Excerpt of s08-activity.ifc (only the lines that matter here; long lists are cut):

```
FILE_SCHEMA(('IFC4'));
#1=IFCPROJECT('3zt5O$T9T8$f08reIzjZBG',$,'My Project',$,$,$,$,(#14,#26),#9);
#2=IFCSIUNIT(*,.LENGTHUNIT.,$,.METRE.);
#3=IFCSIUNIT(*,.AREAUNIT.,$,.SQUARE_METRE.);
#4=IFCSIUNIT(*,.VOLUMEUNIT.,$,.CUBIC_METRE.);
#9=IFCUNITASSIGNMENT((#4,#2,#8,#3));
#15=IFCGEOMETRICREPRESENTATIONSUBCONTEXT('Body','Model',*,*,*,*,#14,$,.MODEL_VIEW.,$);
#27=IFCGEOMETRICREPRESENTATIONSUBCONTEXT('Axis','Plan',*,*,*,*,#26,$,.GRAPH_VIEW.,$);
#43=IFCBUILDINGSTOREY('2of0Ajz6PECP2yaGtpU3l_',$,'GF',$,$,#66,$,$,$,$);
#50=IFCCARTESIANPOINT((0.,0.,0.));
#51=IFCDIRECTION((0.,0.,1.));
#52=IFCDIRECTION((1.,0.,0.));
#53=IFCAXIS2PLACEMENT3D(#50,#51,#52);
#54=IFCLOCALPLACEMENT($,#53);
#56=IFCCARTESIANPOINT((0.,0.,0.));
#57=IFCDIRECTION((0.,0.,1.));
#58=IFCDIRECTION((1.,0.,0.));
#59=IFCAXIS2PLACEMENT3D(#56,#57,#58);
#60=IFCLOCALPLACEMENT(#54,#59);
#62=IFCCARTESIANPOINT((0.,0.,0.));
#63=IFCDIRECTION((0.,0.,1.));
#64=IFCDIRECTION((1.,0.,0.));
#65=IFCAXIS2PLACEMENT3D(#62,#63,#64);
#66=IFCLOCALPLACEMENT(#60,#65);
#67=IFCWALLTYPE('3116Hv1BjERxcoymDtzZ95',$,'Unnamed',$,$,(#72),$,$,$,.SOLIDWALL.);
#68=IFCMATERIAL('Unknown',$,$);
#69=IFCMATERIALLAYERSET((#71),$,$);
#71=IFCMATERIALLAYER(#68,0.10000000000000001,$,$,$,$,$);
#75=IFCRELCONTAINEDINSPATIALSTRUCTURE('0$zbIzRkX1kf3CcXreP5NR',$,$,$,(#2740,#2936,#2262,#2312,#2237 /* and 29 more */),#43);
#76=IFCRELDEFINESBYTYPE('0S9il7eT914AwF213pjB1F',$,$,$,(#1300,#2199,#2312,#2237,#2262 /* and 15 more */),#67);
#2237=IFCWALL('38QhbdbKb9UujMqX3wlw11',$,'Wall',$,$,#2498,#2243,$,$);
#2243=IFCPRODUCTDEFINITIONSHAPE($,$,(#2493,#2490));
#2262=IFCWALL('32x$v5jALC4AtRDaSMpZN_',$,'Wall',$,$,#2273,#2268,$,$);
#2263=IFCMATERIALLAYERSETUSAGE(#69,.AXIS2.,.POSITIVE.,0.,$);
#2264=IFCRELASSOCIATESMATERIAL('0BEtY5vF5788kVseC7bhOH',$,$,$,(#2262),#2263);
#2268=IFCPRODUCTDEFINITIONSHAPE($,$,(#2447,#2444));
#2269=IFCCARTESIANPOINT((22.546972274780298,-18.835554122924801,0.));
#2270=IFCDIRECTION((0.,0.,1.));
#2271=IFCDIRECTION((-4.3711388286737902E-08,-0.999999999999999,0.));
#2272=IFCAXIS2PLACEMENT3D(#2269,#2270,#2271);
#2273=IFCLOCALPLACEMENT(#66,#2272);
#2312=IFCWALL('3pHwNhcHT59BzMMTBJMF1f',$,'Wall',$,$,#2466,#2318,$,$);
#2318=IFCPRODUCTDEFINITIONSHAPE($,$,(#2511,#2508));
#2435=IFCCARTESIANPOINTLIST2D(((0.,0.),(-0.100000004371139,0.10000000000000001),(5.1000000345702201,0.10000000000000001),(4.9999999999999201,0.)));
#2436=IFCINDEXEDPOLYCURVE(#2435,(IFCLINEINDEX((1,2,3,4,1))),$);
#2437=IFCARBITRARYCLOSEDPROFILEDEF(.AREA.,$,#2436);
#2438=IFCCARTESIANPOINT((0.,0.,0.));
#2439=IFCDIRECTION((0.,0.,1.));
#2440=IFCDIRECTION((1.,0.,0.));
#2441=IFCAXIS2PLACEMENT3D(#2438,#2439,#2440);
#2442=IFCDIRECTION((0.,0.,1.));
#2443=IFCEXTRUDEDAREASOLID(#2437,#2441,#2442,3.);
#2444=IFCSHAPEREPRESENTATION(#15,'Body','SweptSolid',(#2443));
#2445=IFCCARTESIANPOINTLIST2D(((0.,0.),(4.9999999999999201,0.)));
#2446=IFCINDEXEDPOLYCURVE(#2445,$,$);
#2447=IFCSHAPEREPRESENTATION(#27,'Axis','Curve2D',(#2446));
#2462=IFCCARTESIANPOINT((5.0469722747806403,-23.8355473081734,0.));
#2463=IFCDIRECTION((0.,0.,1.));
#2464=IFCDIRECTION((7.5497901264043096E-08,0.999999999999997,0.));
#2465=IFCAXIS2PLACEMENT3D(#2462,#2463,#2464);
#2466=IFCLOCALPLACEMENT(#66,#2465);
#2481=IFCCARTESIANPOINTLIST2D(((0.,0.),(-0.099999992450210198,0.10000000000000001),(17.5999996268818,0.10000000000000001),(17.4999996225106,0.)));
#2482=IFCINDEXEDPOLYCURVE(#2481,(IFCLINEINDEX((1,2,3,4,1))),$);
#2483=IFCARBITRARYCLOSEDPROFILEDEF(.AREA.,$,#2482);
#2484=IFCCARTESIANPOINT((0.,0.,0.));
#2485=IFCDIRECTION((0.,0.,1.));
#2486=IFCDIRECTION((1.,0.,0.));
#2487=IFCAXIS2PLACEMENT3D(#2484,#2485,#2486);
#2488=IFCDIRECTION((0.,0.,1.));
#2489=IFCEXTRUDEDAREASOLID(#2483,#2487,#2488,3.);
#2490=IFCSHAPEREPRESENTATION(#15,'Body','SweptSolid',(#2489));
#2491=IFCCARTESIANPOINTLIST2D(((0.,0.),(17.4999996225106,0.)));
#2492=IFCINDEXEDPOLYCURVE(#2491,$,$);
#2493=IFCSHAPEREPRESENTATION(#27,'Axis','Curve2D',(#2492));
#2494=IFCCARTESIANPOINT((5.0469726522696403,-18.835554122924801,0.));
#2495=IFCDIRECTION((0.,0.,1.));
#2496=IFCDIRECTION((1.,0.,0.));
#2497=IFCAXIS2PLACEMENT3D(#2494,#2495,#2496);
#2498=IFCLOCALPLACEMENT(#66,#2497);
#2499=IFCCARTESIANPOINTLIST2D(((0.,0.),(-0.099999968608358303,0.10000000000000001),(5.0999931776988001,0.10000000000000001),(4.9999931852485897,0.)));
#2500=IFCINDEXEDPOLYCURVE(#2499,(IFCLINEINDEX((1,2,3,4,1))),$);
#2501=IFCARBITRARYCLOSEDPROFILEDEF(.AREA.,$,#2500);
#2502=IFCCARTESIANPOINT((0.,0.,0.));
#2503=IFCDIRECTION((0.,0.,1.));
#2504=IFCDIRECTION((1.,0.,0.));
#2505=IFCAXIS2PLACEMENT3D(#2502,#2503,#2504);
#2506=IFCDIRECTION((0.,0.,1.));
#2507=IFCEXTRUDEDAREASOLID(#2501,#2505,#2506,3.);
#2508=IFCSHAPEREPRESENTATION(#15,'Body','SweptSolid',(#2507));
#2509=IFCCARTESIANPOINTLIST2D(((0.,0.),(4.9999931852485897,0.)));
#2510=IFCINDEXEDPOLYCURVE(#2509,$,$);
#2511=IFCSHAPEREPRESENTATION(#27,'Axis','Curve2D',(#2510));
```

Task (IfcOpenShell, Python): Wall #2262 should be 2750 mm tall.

```python
import ifcopenshell
import ifcopenshell.geom
import ifcopenshell.util.representation
import ifcopenshell.util.shape
import ifcopenshell.util.unit

model = ifcopenshell.open("s08-activity.ifc")
unit_scale = ifcopenshell.util.unit.calculate_unit_scale(model)
settings = ifcopenshell.geom.settings()


def volume(element):
    """Net volume in cubic metres, openings subtracted."""
    shape = ifcopenshell.geom.create_shape(settings, element)
    return ifcopenshell.util.shape.get_volume(shape.geometry)


wall = model.by_id(2262)
before = volume(wall)

body = ifcopenshell.util.representation.get_representation(wall, "Model", "Body")
solid = body.Items[0]
old_height = solid.Depth
solid.Depth = 2.75 / unit_scale
after = volume(wall)

print(f"height {old_height:g} -> {solid.Depth:g}, volume {before:.3f} -> {after:.3f} m3")

model.write("s08-activity-out.ifc")
```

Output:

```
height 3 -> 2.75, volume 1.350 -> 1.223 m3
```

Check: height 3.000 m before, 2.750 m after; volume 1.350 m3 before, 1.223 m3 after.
